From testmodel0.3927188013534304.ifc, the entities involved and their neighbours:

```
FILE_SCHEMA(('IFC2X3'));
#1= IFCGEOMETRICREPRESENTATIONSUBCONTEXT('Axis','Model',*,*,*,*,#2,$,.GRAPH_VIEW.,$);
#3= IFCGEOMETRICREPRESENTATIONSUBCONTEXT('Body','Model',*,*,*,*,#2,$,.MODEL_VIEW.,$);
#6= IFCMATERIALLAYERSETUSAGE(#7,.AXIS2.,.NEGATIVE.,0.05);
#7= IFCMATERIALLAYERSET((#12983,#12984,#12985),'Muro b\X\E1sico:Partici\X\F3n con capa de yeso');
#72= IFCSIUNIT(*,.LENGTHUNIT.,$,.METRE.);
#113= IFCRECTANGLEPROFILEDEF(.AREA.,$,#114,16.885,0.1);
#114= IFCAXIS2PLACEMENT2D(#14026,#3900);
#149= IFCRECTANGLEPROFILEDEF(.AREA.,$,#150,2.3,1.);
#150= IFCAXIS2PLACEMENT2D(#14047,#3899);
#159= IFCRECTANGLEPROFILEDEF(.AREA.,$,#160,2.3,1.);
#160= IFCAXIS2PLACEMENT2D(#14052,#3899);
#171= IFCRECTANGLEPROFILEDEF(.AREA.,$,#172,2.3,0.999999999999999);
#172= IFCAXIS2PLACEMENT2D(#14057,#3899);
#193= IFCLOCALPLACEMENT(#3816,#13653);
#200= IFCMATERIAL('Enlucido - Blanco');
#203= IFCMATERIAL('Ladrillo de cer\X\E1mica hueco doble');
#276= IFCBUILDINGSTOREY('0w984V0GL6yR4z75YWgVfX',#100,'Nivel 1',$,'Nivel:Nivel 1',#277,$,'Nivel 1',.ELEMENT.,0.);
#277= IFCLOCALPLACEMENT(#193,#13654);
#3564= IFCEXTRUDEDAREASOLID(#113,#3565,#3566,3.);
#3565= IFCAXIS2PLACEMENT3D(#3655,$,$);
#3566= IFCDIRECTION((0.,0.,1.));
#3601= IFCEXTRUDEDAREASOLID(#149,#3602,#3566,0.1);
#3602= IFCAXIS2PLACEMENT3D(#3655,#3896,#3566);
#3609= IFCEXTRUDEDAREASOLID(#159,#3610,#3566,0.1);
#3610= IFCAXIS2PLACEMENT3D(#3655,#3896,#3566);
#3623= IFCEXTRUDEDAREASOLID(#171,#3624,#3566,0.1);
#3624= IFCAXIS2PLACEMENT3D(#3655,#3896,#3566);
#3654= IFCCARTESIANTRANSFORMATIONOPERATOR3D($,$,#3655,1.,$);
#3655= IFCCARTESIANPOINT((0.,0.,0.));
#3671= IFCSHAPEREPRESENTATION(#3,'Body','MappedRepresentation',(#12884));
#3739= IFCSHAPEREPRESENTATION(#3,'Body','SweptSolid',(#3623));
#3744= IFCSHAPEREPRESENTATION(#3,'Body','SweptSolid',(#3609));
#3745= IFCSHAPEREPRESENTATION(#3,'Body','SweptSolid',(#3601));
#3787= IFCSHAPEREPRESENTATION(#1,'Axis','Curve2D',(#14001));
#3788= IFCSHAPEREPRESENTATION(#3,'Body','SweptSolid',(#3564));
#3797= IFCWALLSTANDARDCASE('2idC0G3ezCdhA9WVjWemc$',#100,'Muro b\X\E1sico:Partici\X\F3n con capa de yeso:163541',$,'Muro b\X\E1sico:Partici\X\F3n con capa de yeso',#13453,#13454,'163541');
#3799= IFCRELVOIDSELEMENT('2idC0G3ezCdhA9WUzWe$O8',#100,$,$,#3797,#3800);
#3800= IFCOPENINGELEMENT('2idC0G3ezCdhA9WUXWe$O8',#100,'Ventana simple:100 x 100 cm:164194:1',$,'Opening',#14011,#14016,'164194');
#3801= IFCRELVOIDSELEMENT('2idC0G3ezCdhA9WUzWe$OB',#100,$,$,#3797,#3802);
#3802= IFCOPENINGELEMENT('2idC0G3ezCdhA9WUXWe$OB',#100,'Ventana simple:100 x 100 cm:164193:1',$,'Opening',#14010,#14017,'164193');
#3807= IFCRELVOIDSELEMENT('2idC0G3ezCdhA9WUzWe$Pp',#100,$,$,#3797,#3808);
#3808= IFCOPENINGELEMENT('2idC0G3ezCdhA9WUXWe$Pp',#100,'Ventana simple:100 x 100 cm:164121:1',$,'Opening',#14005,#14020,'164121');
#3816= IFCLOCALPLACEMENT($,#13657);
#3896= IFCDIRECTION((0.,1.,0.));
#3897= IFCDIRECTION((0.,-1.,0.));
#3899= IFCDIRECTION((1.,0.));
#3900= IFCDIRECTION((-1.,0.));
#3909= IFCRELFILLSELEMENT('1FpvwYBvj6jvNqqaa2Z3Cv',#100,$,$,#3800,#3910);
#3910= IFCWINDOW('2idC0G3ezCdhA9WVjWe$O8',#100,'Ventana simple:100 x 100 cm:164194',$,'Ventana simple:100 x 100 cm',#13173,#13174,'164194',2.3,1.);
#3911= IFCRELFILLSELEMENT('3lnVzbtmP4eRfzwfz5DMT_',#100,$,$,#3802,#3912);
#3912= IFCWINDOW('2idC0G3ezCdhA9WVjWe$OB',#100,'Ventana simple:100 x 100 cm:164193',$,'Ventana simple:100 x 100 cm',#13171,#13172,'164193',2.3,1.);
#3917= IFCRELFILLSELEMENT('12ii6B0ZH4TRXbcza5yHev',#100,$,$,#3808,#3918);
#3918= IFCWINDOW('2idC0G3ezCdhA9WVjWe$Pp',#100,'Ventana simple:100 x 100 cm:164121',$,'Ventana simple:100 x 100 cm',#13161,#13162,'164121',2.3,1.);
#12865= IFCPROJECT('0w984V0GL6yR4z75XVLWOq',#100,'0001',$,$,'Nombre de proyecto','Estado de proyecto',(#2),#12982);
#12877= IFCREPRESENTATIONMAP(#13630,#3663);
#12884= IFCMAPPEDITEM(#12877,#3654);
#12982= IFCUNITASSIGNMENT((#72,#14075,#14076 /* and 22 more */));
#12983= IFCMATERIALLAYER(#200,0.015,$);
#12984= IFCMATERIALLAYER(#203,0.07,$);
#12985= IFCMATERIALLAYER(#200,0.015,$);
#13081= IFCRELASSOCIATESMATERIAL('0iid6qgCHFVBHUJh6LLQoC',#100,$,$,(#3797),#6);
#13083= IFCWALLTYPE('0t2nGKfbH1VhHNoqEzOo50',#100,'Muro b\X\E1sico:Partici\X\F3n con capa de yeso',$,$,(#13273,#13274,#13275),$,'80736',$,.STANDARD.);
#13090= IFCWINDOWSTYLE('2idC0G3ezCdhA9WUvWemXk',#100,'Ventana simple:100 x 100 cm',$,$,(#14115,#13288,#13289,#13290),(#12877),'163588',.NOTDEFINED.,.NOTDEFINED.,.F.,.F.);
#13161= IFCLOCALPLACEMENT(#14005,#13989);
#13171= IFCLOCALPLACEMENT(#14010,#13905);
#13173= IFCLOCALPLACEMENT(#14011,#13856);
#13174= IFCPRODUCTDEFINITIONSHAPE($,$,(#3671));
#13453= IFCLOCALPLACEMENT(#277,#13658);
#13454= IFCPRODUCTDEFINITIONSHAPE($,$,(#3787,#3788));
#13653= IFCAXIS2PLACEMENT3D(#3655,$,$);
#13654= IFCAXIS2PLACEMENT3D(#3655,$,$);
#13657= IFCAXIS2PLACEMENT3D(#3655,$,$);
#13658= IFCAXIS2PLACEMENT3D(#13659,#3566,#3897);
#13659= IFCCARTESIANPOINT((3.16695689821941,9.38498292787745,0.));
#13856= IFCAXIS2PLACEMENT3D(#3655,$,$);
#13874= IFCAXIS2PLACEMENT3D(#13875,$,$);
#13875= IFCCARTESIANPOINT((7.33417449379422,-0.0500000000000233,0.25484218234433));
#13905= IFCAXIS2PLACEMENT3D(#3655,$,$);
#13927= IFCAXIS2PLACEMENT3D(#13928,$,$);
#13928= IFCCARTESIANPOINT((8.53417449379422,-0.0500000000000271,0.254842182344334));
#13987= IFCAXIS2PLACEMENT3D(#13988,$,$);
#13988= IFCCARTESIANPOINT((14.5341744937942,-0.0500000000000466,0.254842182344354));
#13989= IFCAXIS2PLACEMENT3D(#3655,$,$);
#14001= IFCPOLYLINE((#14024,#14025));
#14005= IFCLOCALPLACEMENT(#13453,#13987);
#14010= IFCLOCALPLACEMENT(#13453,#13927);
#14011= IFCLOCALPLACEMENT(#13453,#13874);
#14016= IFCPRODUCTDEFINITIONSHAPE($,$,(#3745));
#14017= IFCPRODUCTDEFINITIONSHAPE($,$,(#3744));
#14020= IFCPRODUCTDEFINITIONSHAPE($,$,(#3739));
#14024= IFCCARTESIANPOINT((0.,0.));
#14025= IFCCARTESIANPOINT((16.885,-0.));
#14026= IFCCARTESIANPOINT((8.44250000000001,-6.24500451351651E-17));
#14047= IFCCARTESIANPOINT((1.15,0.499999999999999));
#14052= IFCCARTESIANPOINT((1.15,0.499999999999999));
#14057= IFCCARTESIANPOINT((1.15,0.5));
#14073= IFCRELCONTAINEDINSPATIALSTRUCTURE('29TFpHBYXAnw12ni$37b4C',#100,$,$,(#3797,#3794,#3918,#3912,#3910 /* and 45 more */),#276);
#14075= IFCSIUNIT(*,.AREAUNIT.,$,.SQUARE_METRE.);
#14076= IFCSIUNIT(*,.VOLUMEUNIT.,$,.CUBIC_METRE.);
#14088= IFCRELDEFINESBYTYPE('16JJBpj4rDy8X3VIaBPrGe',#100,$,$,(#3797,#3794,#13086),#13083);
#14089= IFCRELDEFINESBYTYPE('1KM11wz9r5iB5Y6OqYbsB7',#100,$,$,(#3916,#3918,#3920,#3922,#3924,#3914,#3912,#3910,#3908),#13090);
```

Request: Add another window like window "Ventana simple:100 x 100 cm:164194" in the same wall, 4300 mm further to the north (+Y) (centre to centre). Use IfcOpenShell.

```python
import ifcopenshell
import ifcopenshell.api.feature
import ifcopenshell.api.geometry
import ifcopenshell.api.root
import ifcopenshell.geom
import ifcopenshell.util.element
import ifcopenshell.util.placement
import ifcopenshell.util.shape
import ifcopenshell.util.unit

model = ifcopenshell.open("testmodel0.3927188013534304.ifc")
unit_scale = ifcopenshell.util.unit.calculate_unit_scale(model)
settings = ifcopenshell.geom.settings()


def volume(element):
    """Net volume in cubic metres, openings subtracted."""
    shape = ifcopenshell.geom.create_shape(settings, element)
    return ifcopenshell.util.shape.get_volume(shape.geometry)


def reuse_history(source, copy):
    """copy_class also copies each property set's owner history, people and application; keep the originals."""
    for rel in copy.IsDefinedBy:
        if rel.is_a("IfcRelDefinesByProperties") and (history := rel.RelatingPropertyDefinition.OwnerHistory):
            rel.RelatingPropertyDefinition.OwnerHistory = source.OwnerHistory
            ifcopenshell.util.element.remove_deep2(model, history)


window = model.by_guid("2idC0G3ezCdhA9WVjWe$O8")
opening = window.FillsVoids[0].RelatingOpeningElement
wall = opening.VoidsElements[0].RelatingBuildingElement
before = volume(wall)
shift = ifcopenshell.util.placement.get_local_placement(wall.ObjectPlacement)[:3, 0] * -4.3 / unit_scale

# copy_class copies the void relationship, type, container and properties, but no geometry.
new_opening = ifcopenshell.api.root.copy_class(model, product=opening)
new_opening.Representation = ifcopenshell.util.element.copy_deep(
    model, opening.Representation, exclude=["IfcGeometricRepresentationContext", "IfcRepresentationMap"]
)
new_opening.Name = "Ventana simple:100 x 100 cm"
new_opening.Tag = None
new_window = ifcopenshell.api.root.copy_class(model, product=window)
new_window.Representation = ifcopenshell.util.element.copy_deep(
    model, window.Representation, exclude=["IfcGeometricRepresentationContext", "IfcRepresentationMap"]
)
new_window.Name = "Ventana simple:100 x 100 cm"
new_window.Tag = None
reuse_history(window, new_window)
fills = ifcopenshell.api.feature.add_filling(model, opening=new_opening, element=new_window)
fills.OwnerHistory = new_window.OwnerHistory  # required in IFC2X3

for old, new in ((opening, new_opening), (window, new_window)):
    matrix = ifcopenshell.util.placement.get_local_placement(old.ObjectPlacement)
    matrix[:3, 3] += shift
    ifcopenshell.api.geometry.edit_object_placement(model, product=new, matrix=matrix, is_si=False)

after = volume(wall)

print(f"wall volume {before:.3f} -> {after:.3f} m3")

model.write("testmodel0.3927188013534304_edited.ifc")
```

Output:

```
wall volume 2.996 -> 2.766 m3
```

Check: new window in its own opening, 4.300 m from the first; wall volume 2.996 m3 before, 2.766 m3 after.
